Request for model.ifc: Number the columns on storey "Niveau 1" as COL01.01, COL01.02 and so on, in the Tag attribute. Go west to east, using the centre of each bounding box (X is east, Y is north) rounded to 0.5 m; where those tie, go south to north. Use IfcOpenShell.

First a look at what the model holds.

```python
import ifcopenshell
import ifcopenshell.util.element
import ifcopenshell.util.placement

model = ifcopenshell.open("model.ifc")
print(model.schema)
storey = next(s for s in model.by_type("IfcBuildingStorey") if s.Name == "Niveau 1")
columns = [e for e in ifcopenshell.util.element.get_decomposition(storey) if e.is_a("IfcColumn")]
for e in sorted(columns, key=lambda e: e.id()):
    origin = ifcopenshell.util.placement.get_local_placement(e.ObjectPlacement)[:3, 3]
    print(e.id(), e.Tag, e.Name, origin.round(2) + 0.0, sep=" | ")
```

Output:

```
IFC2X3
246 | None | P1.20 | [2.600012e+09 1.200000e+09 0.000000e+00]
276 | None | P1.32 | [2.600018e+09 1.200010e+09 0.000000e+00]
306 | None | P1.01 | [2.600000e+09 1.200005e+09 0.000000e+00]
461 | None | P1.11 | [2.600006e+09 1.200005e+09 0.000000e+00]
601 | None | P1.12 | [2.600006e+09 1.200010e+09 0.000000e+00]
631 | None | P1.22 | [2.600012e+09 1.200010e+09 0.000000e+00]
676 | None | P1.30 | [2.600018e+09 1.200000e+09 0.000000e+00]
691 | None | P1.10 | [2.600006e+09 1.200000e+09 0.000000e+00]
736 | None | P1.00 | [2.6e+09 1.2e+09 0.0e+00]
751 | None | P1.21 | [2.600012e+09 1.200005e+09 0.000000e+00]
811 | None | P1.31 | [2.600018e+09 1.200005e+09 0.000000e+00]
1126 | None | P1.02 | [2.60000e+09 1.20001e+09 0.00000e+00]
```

```python
import ifcopenshell
import ifcopenshell.geom
import ifcopenshell.util.element
import ifcopenshell.util.shape

model = ifcopenshell.open("model.ifc")
settings = ifcopenshell.geom.settings()
settings.set("use-world-coords", True)


def centre(element):
    shape = ifcopenshell.geom.create_shape(settings, element)
    return ifcopenshell.util.shape.get_bbox_centroid(shape.geometry)


storey = next(s for s in model.by_type("IfcBuildingStorey") if s.Name == "Niveau 1")
columns = [e for e in ifcopenshell.util.element.get_decomposition(storey) if e.is_a("IfcColumn")]

# Insertion points can sit at a corner or the storey origin, so sort by the geometry (in metres).
centres = {e: centre(e) for e in columns}
columns.sort(key=lambda e: (round(centres[e][0] / 0.5), centres[e][1]))

for i, e in enumerate(columns, start=1):
    number = f"COL01.{i:02d}"
    e.Tag = number
    print(e.id(), number)

model.write("model_edited.ifc")
```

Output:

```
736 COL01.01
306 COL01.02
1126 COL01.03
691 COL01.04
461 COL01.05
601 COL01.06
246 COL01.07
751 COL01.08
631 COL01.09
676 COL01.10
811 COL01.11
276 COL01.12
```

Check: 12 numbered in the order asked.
